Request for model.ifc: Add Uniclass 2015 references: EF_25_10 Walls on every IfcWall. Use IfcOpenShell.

First a look at what the model holds.

```python
import ifcopenshell

model = ifcopenshell.open("model.ifc")
print(model.schema)
print("classifications:", [c.Name for c in model.by_type("IfcClassification")])
for ifc_class in ("IfcDoor", "IfcRoof", "IfcStair", "IfcWall", "IfcWindow"):
    print(ifc_class, len(model.by_type(ifc_class)))
```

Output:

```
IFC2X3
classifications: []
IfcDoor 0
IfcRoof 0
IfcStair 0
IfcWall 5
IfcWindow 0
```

```python
import ifcopenshell
import ifcopenshell.api.classification

model = ifcopenshell.open("model.ifc")

# IFC2X3 requires Source and Edition and has no link from the project to the system.
system = model.create_entity("IfcClassification", Source="NBS", Edition="2015", Name="Uniclass 2015")

codes = {
    "IfcWall": ("EF_25_10", "Walls"),
}
for ifc_class, (code, name) in codes.items():
    products = model.by_type(ifc_class)
    ifcopenshell.api.classification.add_reference(
        model, products=products, classification=system, identification=code, name=name
    )
    print(code, len(products))

model.write("model_v2.ifc")
```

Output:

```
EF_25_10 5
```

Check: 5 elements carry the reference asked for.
